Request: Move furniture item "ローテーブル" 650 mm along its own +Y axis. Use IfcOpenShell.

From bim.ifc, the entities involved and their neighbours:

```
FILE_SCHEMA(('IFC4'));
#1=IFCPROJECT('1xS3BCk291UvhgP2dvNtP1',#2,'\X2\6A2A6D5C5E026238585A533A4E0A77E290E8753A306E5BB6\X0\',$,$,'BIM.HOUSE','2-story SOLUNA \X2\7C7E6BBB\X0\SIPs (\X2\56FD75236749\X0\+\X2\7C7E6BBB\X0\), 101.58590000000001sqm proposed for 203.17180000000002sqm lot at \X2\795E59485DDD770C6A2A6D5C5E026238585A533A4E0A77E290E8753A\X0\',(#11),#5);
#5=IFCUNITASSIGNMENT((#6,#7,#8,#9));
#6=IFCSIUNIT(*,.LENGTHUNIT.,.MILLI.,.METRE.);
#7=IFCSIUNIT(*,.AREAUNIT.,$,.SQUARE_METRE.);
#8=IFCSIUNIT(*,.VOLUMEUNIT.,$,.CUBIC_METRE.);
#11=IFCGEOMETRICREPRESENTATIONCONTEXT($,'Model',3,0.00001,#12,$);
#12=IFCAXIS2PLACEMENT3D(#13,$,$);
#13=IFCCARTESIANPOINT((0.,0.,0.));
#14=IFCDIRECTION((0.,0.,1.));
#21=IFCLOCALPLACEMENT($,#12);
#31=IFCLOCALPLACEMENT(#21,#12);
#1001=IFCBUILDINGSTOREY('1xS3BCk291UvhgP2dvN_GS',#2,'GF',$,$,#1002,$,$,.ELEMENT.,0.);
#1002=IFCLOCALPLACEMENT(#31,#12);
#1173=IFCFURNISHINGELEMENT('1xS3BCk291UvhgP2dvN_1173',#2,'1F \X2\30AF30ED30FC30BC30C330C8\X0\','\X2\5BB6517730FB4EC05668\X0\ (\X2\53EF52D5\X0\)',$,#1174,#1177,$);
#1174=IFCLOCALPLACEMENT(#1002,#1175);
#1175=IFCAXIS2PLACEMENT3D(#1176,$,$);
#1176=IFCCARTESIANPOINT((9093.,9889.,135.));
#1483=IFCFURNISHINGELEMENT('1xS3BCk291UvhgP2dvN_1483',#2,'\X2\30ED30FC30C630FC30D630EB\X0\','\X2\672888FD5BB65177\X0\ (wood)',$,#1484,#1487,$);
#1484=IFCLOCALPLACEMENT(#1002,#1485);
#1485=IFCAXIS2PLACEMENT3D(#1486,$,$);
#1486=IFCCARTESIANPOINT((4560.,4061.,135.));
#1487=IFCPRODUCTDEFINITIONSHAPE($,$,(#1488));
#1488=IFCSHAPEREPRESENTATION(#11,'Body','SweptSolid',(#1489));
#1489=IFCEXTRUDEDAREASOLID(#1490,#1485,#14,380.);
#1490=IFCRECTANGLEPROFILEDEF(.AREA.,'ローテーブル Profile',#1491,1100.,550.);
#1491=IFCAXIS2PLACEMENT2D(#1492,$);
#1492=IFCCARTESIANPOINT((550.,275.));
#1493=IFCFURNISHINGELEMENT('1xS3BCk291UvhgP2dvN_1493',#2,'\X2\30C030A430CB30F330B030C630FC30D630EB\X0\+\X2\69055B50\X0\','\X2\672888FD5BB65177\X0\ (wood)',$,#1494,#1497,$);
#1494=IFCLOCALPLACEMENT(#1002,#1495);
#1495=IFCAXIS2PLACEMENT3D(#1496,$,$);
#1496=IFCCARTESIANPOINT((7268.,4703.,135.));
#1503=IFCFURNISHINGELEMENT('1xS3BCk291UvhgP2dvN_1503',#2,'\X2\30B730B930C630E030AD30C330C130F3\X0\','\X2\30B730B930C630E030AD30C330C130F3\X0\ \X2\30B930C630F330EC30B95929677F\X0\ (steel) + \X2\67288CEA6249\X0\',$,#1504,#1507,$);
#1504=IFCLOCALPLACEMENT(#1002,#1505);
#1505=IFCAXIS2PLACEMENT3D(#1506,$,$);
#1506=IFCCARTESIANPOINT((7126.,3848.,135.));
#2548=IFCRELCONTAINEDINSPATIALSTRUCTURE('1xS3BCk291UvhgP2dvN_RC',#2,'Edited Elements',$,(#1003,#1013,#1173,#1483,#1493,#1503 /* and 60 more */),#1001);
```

```python
import ifcopenshell
import ifcopenshell.api.geometry
import ifcopenshell.util.placement
import ifcopenshell.util.unit

model = ifcopenshell.open("bim.ifc")
unit_scale = ifcopenshell.util.unit.calculate_unit_scale(model)

item = model.by_guid("1xS3BCk291UvhgP2dvN_1483")
matrix = ifcopenshell.util.placement.get_local_placement(item.ObjectPlacement)
matrix[:3, 3] += matrix[:3, 1] * 0.65 / unit_scale
ifcopenshell.api.geometry.edit_object_placement(model, product=item, matrix=matrix, is_si=False)

print(ifcopenshell.util.placement.get_local_placement(item.ObjectPlacement).round(3) + 0.0)

model.write("bim_edited.ifc")
```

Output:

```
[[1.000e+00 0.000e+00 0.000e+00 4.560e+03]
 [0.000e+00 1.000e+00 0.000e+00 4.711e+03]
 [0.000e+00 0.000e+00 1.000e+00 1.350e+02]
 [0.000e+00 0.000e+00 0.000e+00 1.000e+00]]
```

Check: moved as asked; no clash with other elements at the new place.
